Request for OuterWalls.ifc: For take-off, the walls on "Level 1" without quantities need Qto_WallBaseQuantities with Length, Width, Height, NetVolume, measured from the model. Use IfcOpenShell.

First a look at what the model holds.

```python
import ifcopenshell
import ifcopenshell.util.element
import ifcopenshell.util.unit

model = ifcopenshell.open("OuterWalls.ifc")
print(model.schema)
for unit_type in ("LENGTHUNIT", "AREAUNIT", "VOLUMEUNIT"):
    print(unit_type, ifcopenshell.util.unit.calculate_unit_scale(model, unit_type))
storey = next(s for s in model.by_type("IfcBuildingStorey") if s.Name == "Level 1")
walls = [e for e in ifcopenshell.util.element.get_decomposition(storey) if e.is_a("IfcWall")]
for e in sorted(walls, key=lambda e: e.id()):
    print(e.id(), e.is_a(), e.Name, list(ifcopenshell.util.element.get_psets(e, qtos_only=True)), sep=" | ")
```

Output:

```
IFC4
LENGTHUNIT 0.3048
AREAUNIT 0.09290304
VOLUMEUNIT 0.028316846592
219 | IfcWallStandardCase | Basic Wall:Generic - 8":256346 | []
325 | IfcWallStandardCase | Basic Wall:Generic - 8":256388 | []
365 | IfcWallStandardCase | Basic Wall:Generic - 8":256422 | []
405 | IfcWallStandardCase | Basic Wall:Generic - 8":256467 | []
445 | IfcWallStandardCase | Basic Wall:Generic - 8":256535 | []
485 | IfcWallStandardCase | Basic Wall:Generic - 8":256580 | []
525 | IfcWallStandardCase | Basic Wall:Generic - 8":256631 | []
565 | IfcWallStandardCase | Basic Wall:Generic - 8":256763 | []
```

```python
import ifcopenshell
import ifcopenshell.api.pset
import ifcopenshell.geom
import ifcopenshell.util.element
import ifcopenshell.util.shape
import ifcopenshell.util.unit

model = ifcopenshell.open("OuterWalls.ifc")
unit_scale = ifcopenshell.util.unit.calculate_unit_scale(model)
volume_scale = ifcopenshell.util.unit.calculate_unit_scale(model, "VOLUMEUNIT")
settings = ifcopenshell.geom.settings()

storey = next(s for s in model.by_type("IfcBuildingStorey") if s.Name == "Level 1")
walls = [e for e in ifcopenshell.util.element.get_decomposition(storey) if e.is_a("IfcWall")]

for e in sorted(walls, key=lambda e: e.id()):
    if ifcopenshell.util.element.get_psets(e, qtos_only=True, should_inherit=False):
        continue
    # Geometry comes back in metres, in the element's own axes.
    shape = ifcopenshell.geom.create_shape(settings, e)
    values = {
        "Length": ifcopenshell.util.shape.get_x(shape.geometry) / unit_scale,
        "Width": ifcopenshell.util.shape.get_y(shape.geometry) / unit_scale,
        "Height": ifcopenshell.util.shape.get_z(shape.geometry) / unit_scale,
        "NetVolume": ifcopenshell.util.shape.get_volume(shape.geometry) / volume_scale,
    }
    qto = ifcopenshell.api.pset.add_qto(model, product=e, name="Qto_WallBaseQuantities")
    ifcopenshell.api.pset.edit_qto(model, qto=qto, properties=values)
    print(e.id(), {k: round(v, 3) for k, v in values.items()})

model.write("OuterWalls_v2.ifc")
```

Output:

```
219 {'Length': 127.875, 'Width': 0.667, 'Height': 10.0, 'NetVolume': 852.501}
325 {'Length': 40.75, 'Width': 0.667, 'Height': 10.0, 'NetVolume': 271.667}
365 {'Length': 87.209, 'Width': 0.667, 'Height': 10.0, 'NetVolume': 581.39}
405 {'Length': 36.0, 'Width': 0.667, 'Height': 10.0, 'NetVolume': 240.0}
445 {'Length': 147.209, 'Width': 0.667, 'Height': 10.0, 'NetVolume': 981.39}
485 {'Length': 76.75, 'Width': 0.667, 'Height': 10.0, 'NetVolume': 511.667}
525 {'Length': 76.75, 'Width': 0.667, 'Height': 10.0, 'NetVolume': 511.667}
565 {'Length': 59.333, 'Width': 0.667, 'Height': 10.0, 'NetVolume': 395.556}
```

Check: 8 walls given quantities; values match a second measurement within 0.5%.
